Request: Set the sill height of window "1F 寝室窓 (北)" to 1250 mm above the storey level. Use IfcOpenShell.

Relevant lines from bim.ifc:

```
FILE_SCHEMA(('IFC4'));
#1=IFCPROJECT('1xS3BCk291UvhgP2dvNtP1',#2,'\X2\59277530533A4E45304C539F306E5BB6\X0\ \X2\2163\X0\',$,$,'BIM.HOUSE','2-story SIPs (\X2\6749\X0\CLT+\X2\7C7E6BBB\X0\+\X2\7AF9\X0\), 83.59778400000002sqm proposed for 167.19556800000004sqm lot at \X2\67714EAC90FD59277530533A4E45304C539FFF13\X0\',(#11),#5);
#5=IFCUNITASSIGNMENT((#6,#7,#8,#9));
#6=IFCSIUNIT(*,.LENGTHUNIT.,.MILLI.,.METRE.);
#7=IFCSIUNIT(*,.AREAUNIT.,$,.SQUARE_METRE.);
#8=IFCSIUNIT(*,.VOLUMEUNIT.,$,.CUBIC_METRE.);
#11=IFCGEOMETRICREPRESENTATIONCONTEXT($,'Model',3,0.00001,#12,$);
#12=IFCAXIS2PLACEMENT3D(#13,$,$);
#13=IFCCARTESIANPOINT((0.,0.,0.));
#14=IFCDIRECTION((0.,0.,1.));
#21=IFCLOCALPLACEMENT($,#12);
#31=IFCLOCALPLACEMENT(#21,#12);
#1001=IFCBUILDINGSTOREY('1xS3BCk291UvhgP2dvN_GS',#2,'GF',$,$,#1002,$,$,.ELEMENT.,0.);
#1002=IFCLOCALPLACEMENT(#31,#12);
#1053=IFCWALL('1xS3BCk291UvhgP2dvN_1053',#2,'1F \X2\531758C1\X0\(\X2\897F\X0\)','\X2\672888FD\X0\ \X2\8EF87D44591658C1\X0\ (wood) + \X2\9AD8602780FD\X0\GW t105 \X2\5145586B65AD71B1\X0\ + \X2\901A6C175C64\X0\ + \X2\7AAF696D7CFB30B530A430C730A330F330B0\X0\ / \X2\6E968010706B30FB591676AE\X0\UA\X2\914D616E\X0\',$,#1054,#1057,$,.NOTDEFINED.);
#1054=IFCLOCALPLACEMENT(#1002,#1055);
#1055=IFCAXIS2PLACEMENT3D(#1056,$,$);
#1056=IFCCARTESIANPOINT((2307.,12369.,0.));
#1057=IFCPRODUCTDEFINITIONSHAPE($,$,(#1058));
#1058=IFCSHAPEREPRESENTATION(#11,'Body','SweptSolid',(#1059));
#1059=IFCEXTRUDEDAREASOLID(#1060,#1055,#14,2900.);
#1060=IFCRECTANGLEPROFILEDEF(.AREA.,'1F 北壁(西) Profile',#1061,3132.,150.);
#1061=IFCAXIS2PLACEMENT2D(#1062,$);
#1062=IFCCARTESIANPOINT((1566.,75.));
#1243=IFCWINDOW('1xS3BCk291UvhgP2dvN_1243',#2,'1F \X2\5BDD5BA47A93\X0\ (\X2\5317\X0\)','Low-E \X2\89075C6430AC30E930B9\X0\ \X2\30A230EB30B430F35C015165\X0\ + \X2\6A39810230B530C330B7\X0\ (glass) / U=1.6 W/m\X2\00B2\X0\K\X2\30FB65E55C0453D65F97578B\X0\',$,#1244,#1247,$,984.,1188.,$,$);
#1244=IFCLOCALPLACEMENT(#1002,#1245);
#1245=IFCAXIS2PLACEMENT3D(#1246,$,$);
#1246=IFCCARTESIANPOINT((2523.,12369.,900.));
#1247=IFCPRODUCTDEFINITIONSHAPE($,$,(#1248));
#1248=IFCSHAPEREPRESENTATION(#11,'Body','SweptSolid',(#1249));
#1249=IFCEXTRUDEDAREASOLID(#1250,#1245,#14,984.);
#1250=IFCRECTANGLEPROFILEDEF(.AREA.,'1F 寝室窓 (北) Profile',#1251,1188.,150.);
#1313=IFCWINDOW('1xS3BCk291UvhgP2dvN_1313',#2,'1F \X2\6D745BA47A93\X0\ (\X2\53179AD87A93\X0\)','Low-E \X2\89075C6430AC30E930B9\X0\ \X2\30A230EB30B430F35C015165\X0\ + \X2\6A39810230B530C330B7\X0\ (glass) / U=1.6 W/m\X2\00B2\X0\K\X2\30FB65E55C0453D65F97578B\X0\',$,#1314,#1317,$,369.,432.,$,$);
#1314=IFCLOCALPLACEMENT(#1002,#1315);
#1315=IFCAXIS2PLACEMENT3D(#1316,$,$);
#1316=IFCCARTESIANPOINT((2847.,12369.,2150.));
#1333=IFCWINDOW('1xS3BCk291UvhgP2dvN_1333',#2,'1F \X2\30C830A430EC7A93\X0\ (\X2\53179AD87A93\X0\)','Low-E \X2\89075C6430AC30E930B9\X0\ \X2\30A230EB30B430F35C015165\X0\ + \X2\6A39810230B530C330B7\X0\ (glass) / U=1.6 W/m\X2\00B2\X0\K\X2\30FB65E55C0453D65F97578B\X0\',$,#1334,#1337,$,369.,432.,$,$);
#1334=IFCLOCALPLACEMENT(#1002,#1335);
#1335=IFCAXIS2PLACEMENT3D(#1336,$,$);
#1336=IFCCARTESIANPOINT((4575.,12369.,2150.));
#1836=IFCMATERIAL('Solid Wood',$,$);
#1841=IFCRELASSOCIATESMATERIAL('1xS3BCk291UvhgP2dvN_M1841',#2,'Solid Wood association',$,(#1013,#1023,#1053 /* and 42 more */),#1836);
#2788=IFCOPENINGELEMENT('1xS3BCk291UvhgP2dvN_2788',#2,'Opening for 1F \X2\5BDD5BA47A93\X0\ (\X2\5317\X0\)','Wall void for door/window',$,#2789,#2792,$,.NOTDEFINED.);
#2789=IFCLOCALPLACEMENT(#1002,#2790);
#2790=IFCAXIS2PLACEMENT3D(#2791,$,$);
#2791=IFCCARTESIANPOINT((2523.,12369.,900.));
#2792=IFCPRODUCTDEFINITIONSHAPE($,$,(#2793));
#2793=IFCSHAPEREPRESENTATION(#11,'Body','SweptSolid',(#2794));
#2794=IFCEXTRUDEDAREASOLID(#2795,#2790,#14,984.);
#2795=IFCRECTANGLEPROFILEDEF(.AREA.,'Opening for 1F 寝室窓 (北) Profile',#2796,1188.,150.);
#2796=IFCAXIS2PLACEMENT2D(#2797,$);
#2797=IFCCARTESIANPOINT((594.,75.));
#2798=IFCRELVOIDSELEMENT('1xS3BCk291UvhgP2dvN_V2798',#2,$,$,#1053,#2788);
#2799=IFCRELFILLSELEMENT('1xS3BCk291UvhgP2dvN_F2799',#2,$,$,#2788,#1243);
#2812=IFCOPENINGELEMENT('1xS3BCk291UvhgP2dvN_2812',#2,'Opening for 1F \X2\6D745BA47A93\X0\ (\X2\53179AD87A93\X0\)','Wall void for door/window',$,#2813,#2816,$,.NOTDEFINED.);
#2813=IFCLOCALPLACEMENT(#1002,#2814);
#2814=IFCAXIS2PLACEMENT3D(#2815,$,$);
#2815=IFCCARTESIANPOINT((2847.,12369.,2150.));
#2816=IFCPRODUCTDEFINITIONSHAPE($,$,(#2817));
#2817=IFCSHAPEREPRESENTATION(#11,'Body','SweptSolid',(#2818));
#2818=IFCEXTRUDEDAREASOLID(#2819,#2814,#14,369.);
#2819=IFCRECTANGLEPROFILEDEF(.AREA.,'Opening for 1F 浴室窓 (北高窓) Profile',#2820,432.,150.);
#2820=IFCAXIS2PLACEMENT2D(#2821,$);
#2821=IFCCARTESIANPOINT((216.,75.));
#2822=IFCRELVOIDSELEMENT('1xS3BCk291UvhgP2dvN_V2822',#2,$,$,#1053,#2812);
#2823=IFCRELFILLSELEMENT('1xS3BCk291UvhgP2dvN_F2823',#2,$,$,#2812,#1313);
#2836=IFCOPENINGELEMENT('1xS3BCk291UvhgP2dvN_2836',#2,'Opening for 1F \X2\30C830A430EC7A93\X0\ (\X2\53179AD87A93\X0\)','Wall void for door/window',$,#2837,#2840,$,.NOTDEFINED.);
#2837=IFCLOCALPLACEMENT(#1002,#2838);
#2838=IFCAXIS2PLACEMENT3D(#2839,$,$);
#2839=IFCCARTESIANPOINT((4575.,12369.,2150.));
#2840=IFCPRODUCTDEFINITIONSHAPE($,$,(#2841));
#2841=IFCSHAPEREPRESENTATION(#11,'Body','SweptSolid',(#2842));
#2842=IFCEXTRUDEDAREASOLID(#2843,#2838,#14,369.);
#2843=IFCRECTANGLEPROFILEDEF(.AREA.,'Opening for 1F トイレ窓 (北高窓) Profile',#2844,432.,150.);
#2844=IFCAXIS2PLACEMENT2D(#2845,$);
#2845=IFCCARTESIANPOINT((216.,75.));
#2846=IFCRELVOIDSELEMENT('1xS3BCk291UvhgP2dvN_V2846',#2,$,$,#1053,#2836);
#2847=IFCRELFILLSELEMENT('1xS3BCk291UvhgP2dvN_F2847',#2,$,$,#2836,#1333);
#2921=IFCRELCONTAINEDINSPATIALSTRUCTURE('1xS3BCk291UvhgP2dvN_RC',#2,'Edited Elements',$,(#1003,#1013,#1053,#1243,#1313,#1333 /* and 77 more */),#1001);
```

```python
import numpy as np
import ifcopenshell
import ifcopenshell.api.geometry
import ifcopenshell.geom
import ifcopenshell.util.element
import ifcopenshell.util.placement
import ifcopenshell.util.shape
import ifcopenshell.util.unit

model = ifcopenshell.open("bim.ifc")
unit_scale = ifcopenshell.util.unit.calculate_unit_scale(model)

window = model.by_id(1243)
opening = window.FillsVoids[0].RelatingOpeningElement
storey = ifcopenshell.util.element.get_container(window, ifc_class="IfcBuildingStorey")
level = ifcopenshell.util.placement.get_local_placement(storey.ObjectPlacement)[2, 3]

# The opening's origin need not be at the sill, so measure its lowest point.
shape = ifcopenshell.geom.create_shape(ifcopenshell.geom.settings(), opening)
bottom = ifcopenshell.util.shape.get_shape_bottom_elevation(shape, shape.geometry) / unit_scale
dz = level + 1250.0 - bottom

shift = np.array([0.0, 0.0, dz])
# The window is not placed relative to its opening, so move both.
for product in (opening, window):
    matrix = ifcopenshell.util.placement.get_local_placement(product.ObjectPlacement)
    matrix[:3, 3] += shift
    ifcopenshell.api.geometry.edit_object_placement(model, product=product, matrix=matrix, is_si=False)

print(f"moved by {dz * unit_scale:+.3f} m")

model.write("bim_rev.ifc")
```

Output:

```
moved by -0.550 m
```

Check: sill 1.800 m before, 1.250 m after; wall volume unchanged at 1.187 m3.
